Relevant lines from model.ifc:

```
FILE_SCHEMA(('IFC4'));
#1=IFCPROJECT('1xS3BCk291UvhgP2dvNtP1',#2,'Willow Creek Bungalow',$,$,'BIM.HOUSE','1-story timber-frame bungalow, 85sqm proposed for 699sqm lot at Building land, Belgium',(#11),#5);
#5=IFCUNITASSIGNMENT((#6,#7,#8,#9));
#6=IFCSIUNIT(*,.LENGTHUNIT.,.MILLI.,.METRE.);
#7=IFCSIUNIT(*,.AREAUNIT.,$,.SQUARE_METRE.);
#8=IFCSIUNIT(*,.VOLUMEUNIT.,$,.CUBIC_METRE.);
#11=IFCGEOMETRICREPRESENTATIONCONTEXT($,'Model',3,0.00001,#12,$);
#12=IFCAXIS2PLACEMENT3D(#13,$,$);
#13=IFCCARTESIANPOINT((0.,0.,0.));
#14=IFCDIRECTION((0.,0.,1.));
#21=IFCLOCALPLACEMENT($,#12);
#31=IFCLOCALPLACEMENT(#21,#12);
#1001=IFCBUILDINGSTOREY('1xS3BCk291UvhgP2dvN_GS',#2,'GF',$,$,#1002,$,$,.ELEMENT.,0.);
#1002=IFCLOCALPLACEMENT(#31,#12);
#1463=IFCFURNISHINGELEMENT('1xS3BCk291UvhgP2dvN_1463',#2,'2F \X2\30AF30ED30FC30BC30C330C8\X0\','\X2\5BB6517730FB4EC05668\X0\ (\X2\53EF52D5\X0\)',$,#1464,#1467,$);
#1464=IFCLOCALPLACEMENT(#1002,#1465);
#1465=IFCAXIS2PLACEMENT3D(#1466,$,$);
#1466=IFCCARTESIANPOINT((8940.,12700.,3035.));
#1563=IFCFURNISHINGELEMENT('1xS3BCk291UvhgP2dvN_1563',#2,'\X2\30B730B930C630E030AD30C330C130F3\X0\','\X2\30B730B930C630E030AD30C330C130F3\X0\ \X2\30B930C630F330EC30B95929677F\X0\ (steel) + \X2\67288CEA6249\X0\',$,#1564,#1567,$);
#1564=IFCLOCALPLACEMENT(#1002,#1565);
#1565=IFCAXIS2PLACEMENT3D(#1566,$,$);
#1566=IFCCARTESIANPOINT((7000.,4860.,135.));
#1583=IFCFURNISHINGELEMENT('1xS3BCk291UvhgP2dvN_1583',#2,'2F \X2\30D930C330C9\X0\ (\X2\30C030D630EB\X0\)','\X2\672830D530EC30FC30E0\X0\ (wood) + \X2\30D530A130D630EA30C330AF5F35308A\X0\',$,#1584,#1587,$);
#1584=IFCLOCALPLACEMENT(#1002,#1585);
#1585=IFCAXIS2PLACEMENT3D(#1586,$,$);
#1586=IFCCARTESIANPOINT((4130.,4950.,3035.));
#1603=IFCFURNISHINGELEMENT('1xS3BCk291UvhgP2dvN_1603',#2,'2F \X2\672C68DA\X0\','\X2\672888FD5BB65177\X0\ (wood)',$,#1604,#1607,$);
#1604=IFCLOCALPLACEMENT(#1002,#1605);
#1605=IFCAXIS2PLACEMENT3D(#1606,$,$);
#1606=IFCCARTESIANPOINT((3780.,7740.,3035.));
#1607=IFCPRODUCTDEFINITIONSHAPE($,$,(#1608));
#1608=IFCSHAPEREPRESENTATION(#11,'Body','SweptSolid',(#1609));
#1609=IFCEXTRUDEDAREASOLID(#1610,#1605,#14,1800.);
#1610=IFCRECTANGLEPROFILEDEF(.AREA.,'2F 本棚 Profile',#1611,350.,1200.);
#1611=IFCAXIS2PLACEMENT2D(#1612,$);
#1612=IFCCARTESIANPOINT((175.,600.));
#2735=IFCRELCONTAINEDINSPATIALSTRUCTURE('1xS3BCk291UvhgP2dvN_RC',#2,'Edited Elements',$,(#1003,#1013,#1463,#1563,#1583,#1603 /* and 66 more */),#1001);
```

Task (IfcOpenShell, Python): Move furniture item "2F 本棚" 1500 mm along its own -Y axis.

```python
import ifcopenshell
import ifcopenshell.api.geometry
import ifcopenshell.util.placement
import ifcopenshell.util.unit

model = ifcopenshell.open("model.ifc")
unit_scale = ifcopenshell.util.unit.calculate_unit_scale(model)

item = model.by_guid("1xS3BCk291UvhgP2dvN_1603")
matrix = ifcopenshell.util.placement.get_local_placement(item.ObjectPlacement)
matrix[:3, 3] -= matrix[:3, 1] * 1.5 / unit_scale
ifcopenshell.api.geometry.edit_object_placement(model, product=item, matrix=matrix, is_si=False)

print(ifcopenshell.util.placement.get_local_placement(item.ObjectPlacement).round(3) + 0.0)

model.write("model_updated.ifc")
```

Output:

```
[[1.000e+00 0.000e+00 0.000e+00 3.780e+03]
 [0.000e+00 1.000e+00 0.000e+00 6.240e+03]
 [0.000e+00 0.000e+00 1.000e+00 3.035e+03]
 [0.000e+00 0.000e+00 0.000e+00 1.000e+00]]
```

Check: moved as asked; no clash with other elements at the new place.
